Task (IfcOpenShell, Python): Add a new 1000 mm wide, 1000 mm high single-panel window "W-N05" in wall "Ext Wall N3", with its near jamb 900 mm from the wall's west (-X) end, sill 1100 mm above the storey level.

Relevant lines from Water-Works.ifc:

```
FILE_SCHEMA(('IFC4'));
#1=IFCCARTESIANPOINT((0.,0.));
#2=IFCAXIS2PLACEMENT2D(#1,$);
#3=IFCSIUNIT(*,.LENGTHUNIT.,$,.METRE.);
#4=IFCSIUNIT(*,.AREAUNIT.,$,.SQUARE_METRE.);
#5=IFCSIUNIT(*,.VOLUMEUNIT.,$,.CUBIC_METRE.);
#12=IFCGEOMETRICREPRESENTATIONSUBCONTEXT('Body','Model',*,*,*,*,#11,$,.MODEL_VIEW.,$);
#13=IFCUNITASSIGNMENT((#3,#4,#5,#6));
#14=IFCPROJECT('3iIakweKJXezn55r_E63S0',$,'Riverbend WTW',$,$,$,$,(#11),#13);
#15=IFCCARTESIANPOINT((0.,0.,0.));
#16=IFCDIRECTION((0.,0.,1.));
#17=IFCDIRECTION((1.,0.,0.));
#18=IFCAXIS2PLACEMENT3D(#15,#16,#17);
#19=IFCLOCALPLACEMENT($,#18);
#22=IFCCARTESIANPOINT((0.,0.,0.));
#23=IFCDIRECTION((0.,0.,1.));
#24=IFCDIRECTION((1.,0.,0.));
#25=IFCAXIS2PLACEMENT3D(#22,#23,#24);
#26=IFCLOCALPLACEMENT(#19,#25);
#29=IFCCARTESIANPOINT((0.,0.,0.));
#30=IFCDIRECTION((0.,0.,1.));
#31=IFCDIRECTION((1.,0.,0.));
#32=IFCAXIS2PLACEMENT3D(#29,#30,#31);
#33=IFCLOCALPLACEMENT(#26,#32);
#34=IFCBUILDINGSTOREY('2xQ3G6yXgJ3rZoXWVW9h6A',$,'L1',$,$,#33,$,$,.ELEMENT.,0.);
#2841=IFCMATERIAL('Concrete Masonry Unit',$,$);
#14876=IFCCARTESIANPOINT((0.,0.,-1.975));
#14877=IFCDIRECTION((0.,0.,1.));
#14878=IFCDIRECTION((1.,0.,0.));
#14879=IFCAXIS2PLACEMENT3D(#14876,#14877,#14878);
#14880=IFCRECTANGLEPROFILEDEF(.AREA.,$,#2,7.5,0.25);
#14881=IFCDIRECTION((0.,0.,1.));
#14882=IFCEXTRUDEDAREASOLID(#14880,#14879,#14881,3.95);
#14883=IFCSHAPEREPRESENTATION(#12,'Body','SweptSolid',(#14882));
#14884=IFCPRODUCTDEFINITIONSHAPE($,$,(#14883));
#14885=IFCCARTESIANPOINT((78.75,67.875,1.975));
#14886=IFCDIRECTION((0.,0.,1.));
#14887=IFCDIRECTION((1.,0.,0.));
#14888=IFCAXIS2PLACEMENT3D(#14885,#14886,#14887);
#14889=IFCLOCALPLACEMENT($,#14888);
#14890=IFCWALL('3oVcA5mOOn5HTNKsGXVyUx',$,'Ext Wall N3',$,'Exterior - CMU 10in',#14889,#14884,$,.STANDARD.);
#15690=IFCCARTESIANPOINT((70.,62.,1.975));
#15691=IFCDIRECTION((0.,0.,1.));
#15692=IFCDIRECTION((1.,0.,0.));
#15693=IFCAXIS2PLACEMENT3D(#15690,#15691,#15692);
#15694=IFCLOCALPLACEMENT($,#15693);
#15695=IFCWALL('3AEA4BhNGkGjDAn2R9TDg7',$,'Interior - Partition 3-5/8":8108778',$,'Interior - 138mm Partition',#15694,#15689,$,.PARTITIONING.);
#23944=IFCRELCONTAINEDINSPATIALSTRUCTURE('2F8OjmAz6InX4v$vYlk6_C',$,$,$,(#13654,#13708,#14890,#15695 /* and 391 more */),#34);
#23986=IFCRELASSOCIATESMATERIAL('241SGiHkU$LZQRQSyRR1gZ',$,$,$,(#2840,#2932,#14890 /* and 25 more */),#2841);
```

```python
import numpy as np
import ifcopenshell
import ifcopenshell.api.feature
import ifcopenshell.api.geometry
import ifcopenshell.api.root
import ifcopenshell.api.spatial
import ifcopenshell.geom
import ifcopenshell.util.element
import ifcopenshell.util.placement
import ifcopenshell.util.representation
import ifcopenshell.util.shape
import ifcopenshell.util.unit

model = ifcopenshell.open("Water-Works.ifc")
unit_scale = ifcopenshell.util.unit.calculate_unit_scale(model)
settings = ifcopenshell.geom.settings()


def volume(element):
    """Net volume in cubic metres, openings subtracted."""
    shape = ifcopenshell.geom.create_shape(settings, element)
    return ifcopenshell.util.shape.get_volume(shape.geometry)


wall = model.by_id(14890)
storey = ifcopenshell.util.element.get_container(wall, ifc_class="IfcBuildingStorey")
context = ifcopenshell.util.representation.get_context(model, "Model", "Body", "MODEL_VIEW")
before = volume(wall)

width, height, from_end, sill = 1, 1, 0.9, 1.1  # metres

# The wall runs along its own X axis, and the end named is its -X end.
wall_shape = ifcopenshell.geom.create_shape(settings, wall)
x, y, z = ifcopenshell.util.shape.get_vertices(wall_shape.geometry).T
start = x.min() + from_end
face, thickness = float(y.min()), float(y.max() - y.min())
wall_matrix = ifcopenshell.util.placement.get_local_placement(wall.ObjectPlacement)
level = ifcopenshell.util.placement.get_local_placement(storey.ObjectPlacement)[2, 3]


def in_wall(x, y):
    """Placement at x, y metres in the wall's axes, at sill height."""
    matrix = wall_matrix.copy()
    matrix[:, 3] = wall_matrix @ np.array([x / unit_scale, y / unit_scale, 0.0, 1.0])
    matrix[2, 3] = level + sill / unit_scale
    return matrix


# Opening: a box that overshoots both wall faces by 50 mm.
opening = ifcopenshell.api.root.create_entity(model, ifc_class="IfcOpeningElement", predefined_type="OPENING")
box = ifcopenshell.api.geometry.add_wall_representation(
    model, context=context, length=width, height=height, thickness=thickness + 0.1
)
ifcopenshell.api.geometry.assign_representation(model, product=opening, representation=box)
ifcopenshell.api.geometry.edit_object_placement(model, product=opening, matrix=in_wall(start, face - 0.05), is_si=False)
ifcopenshell.api.feature.add_feature(model, feature=opening, element=wall)

window = ifcopenshell.api.root.create_entity(model, ifc_class="IfcWindow", name="W-N05", predefined_type="WINDOW")
window.OverallWidth, window.OverallHeight = width / unit_scale, height / unit_scale
window.PartitioningType = "SINGLE_PANEL"
body = ifcopenshell.api.geometry.add_window_representation(
    model,
    context=context,
    overall_width=window.OverallWidth,
    overall_height=window.OverallHeight,
    partition_type="SINGLE_PANEL",
)
ifcopenshell.api.geometry.assign_representation(model, product=window, representation=body)
ifcopenshell.api.spatial.assign_container(model, products=[window], relating_structure=storey)
ifcopenshell.api.feature.add_filling(model, opening=opening, element=window)

# Centre the window in the wall's thickness.
ifcopenshell.api.geometry.edit_object_placement(model, product=window, matrix=in_wall(start, face), is_si=False)
window_shape = ifcopenshell.geom.create_shape(settings, window)
depth = ifcopenshell.util.shape.get_vertices(window_shape.geometry)[:, 1]
offset = face + thickness / 2 - (depth.min() + depth.max()) / 2
ifcopenshell.api.geometry.edit_object_placement(model, product=window, matrix=in_wall(start, offset), is_si=False)

after = volume(wall)

print(f"wall volume {before:.3f} -> {after:.3f} m3")

model.write("Water-Works_rev.ifc")
```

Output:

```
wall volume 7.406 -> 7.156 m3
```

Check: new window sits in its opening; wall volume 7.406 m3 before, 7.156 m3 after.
